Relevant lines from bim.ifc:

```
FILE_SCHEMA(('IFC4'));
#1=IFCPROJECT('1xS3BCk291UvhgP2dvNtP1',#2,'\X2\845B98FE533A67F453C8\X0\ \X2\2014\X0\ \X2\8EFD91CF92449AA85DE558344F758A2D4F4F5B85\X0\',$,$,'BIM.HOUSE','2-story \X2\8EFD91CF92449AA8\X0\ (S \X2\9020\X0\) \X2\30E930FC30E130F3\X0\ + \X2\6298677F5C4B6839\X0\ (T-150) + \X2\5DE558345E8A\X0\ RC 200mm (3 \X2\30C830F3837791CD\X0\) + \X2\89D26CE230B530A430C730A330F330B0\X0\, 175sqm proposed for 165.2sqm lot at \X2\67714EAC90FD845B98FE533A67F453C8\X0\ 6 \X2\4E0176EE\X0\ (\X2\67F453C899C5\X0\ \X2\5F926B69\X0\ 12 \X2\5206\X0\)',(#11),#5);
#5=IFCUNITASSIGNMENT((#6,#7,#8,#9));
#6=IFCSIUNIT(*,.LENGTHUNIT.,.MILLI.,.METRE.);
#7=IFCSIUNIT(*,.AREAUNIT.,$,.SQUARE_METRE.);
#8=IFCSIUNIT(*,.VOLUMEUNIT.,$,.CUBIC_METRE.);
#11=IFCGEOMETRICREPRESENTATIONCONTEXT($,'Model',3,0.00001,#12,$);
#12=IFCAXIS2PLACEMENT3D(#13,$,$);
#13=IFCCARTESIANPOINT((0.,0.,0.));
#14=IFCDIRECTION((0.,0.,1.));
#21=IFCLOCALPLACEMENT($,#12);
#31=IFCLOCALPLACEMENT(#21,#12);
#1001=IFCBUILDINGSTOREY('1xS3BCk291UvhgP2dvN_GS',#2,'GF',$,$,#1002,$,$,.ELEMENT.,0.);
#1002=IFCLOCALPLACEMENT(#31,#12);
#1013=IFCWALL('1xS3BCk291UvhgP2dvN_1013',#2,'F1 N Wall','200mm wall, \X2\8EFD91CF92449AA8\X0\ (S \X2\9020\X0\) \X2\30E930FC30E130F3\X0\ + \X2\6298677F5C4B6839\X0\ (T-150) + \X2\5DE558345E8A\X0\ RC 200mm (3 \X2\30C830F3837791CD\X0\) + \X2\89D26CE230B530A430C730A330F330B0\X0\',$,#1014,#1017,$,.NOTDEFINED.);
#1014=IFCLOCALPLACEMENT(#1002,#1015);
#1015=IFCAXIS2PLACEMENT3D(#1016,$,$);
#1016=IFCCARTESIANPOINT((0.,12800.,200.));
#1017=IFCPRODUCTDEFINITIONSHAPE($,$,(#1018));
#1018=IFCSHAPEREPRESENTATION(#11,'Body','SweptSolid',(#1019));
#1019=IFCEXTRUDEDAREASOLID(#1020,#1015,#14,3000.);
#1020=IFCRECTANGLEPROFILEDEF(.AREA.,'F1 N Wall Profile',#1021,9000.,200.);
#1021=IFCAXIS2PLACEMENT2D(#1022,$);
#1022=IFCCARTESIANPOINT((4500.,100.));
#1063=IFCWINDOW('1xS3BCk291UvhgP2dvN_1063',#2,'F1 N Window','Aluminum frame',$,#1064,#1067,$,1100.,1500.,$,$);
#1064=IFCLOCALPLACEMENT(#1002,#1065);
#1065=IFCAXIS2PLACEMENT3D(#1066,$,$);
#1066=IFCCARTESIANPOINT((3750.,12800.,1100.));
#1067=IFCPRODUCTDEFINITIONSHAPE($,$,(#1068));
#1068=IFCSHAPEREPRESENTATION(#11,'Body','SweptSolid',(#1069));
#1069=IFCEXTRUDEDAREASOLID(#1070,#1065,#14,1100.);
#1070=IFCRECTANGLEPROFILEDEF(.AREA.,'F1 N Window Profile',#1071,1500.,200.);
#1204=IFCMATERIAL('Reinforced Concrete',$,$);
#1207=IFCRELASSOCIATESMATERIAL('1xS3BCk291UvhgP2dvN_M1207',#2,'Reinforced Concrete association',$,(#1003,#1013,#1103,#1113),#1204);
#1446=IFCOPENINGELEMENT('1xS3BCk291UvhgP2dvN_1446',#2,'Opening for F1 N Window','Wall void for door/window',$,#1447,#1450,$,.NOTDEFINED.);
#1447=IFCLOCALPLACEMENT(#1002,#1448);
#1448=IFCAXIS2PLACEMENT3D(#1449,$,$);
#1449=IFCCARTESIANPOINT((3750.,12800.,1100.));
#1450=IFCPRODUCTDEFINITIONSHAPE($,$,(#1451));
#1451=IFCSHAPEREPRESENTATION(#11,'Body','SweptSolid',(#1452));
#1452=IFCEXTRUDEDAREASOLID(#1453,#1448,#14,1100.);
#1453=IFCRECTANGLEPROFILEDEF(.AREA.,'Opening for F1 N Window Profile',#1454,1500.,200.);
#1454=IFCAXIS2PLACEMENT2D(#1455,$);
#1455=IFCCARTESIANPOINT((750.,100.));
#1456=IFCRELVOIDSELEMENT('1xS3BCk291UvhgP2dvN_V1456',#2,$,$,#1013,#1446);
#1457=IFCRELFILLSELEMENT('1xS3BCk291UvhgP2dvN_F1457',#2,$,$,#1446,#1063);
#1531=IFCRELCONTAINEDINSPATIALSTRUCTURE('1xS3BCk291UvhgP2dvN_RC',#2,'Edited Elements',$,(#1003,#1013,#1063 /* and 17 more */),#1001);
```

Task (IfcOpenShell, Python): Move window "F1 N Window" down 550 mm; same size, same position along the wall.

```python
import numpy as np
import ifcopenshell
import ifcopenshell.api.geometry
import ifcopenshell.util.placement
import ifcopenshell.util.unit

model = ifcopenshell.open("bim.ifc")
unit_scale = ifcopenshell.util.unit.calculate_unit_scale(model)

window = model.by_guid("1xS3BCk291UvhgP2dvN_1063")
opening = window.FillsVoids[0].RelatingOpeningElement
dz = -0.55 / unit_scale

shift = np.array([0.0, 0.0, dz])
# The window is not placed relative to its opening, so move both.
for product in (opening, window):
    matrix = ifcopenshell.util.placement.get_local_placement(product.ObjectPlacement)
    matrix[:3, 3] += shift
    ifcopenshell.api.geometry.edit_object_placement(model, product=product, matrix=matrix, is_si=False)

print(f"moved by {dz * unit_scale:+.3f} m")

model.write("bim_rev.ifc")
```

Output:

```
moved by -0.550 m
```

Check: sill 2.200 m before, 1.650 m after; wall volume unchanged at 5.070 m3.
